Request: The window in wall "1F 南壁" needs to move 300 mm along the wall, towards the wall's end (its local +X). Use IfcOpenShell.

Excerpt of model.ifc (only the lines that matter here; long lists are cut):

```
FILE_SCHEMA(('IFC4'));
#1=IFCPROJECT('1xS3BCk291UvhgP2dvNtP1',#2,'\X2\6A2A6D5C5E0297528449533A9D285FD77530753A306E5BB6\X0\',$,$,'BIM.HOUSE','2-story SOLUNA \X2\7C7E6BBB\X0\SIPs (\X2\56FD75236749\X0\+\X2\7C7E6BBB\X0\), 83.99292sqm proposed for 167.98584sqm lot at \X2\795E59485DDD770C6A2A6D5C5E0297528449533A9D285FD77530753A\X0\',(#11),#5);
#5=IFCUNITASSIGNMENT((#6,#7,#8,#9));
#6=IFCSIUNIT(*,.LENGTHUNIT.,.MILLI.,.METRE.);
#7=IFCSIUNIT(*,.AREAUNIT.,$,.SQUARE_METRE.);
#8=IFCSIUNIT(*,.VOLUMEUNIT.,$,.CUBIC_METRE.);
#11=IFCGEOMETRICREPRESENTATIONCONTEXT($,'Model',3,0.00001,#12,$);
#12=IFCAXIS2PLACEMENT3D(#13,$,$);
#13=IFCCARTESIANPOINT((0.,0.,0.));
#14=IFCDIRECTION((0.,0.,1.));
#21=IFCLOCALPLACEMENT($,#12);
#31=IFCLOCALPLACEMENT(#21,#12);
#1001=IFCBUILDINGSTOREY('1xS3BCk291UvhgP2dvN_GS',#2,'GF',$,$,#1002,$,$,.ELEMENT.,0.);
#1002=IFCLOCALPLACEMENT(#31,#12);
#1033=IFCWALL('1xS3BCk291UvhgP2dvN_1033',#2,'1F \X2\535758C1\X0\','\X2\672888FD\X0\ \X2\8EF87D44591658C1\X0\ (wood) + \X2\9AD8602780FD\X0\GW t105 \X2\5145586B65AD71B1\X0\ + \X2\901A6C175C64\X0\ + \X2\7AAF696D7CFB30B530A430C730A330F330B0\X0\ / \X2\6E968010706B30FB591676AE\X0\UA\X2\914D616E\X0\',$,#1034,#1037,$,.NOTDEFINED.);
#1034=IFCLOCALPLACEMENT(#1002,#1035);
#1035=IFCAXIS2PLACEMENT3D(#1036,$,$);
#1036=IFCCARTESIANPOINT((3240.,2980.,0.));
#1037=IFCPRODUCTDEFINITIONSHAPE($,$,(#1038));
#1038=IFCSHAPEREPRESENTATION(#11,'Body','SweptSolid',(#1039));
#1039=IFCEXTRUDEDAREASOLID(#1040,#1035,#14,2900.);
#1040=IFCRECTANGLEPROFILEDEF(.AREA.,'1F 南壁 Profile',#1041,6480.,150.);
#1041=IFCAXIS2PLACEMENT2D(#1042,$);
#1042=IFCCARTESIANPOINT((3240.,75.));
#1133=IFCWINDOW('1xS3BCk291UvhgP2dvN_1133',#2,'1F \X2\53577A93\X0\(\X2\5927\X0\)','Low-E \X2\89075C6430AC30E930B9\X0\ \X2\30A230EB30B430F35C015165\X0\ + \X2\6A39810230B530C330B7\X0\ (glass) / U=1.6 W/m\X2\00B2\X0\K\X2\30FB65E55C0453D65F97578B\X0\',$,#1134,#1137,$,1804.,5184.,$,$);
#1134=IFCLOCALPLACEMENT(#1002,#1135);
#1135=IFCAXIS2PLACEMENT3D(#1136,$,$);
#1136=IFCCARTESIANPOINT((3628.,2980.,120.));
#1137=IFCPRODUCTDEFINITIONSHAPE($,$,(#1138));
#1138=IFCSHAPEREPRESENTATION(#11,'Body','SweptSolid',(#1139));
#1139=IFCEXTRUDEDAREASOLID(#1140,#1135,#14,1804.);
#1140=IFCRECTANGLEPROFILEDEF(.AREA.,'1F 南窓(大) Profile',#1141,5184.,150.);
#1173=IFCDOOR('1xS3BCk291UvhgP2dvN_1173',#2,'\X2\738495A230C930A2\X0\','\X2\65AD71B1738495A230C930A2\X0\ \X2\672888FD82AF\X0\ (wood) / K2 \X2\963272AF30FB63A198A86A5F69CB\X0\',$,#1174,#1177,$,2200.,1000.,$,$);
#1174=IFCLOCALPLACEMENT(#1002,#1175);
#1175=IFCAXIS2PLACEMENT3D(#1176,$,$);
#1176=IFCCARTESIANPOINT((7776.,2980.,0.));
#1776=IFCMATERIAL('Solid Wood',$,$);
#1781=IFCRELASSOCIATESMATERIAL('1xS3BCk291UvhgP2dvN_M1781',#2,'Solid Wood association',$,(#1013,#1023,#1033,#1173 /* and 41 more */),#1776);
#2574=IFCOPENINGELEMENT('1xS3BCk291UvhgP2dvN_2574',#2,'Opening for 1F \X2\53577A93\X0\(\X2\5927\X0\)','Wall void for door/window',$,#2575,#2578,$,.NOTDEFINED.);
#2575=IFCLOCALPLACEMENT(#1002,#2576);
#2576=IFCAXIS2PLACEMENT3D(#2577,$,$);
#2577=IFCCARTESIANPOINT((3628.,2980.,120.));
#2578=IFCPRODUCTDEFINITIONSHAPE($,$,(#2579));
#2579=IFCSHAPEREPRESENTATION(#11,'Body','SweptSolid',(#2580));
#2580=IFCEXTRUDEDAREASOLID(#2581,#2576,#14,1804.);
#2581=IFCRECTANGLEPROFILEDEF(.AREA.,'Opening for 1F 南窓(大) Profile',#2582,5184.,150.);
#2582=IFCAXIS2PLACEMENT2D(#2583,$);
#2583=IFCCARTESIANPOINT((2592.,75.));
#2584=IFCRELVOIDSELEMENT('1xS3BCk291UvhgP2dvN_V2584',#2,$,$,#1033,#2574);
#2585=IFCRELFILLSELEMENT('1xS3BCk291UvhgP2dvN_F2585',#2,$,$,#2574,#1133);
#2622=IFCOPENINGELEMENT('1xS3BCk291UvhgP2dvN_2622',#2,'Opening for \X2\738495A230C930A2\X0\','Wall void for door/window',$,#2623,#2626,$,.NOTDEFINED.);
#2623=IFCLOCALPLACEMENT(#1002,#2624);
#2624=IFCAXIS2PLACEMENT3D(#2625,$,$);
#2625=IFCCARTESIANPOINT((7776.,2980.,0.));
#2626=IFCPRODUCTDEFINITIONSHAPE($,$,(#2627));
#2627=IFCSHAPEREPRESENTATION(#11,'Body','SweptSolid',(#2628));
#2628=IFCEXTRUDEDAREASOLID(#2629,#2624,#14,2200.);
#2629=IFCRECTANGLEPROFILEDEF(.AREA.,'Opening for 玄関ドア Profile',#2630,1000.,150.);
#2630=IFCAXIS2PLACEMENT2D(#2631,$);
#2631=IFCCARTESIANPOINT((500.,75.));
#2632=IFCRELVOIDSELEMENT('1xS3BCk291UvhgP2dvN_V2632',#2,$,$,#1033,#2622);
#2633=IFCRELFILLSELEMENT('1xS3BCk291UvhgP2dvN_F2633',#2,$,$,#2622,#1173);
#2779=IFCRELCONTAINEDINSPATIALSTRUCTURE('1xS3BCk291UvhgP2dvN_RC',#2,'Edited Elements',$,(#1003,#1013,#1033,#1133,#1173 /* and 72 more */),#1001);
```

```python
import ifcopenshell
import ifcopenshell.api.geometry
import ifcopenshell.util.placement

model = ifcopenshell.open("model.ifc")

window = model.by_id(1133)
opening = window.FillsVoids[0].RelatingOpeningElement
wall = opening.VoidsElements[0].RelatingBuildingElement

wall_matrix = ifcopenshell.util.placement.get_local_placement(wall.ObjectPlacement)
shift = wall_matrix[:3, 0] * 300.0
before = ifcopenshell.util.placement.get_local_placement(window.ObjectPlacement)[:3, 3].copy()

# The window is not placed relative to its opening, so move both.
for product in (opening, window):
    matrix = ifcopenshell.util.placement.get_local_placement(product.ObjectPlacement)
    matrix[:3, 3] += shift
    ifcopenshell.api.geometry.edit_object_placement(model, product=product, matrix=matrix, is_si=False)

after = ifcopenshell.util.placement.get_local_placement(window.ObjectPlacement)[:3, 3]
print("window moved by", (after - before).round(3) + 0.0)

model.write("model_updated.ifc")
```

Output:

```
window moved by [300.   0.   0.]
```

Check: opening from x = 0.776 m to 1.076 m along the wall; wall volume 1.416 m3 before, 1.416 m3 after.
